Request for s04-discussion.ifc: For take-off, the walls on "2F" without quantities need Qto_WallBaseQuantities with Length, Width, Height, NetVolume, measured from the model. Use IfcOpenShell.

First a look at what the model holds.

```python
import ifcopenshell
import ifcopenshell.util.element
import ifcopenshell.util.unit

model = ifcopenshell.open("s04-discussion.ifc")
print(model.schema)
for unit_type in ("LENGTHUNIT", "AREAUNIT", "VOLUMEUNIT"):
    print(unit_type, ifcopenshell.util.unit.calculate_unit_scale(model, unit_type))
storey = next(s for s in model.by_type("IfcBuildingStorey") if s.Name == "2F")
walls = [e for e in ifcopenshell.util.element.get_decomposition(storey) if e.is_a("IfcWall")]
for e in sorted(walls, key=lambda e: e.id()):
    print(e.id(), e.is_a(), e.Name, list(ifcopenshell.util.element.get_psets(e, qtos_only=True)), sep=" | ")
```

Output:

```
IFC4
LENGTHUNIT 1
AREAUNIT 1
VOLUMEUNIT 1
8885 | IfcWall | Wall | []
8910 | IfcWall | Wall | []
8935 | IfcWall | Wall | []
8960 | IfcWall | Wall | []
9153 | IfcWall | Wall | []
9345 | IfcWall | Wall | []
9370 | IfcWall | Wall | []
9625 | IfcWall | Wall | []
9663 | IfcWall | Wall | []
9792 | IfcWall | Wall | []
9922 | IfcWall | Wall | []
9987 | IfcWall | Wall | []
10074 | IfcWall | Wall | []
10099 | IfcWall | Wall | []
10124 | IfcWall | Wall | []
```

```python
import ifcopenshell
import ifcopenshell.api.pset
import ifcopenshell.geom
import ifcopenshell.util.element
import ifcopenshell.util.shape
import ifcopenshell.util.unit

model = ifcopenshell.open("s04-discussion.ifc")
unit_scale = ifcopenshell.util.unit.calculate_unit_scale(model)
volume_scale = ifcopenshell.util.unit.calculate_unit_scale(model, "VOLUMEUNIT")
settings = ifcopenshell.geom.settings()

storey = next(s for s in model.by_type("IfcBuildingStorey") if s.Name == "2F")
walls = [e for e in ifcopenshell.util.element.get_decomposition(storey) if e.is_a("IfcWall")]

for e in sorted(walls, key=lambda e: e.id()):
    if ifcopenshell.util.element.get_psets(e, qtos_only=True, should_inherit=False):
        continue
    # Geometry comes back in metres, in the element's own axes.
    shape = ifcopenshell.geom.create_shape(settings, e)
    values = {
        "Length": ifcopenshell.util.shape.get_x(shape.geometry) / unit_scale,
        "Width": ifcopenshell.util.shape.get_y(shape.geometry) / unit_scale,
        "Height": ifcopenshell.util.shape.get_z(shape.geometry) / unit_scale,
        "NetVolume": ifcopenshell.util.shape.get_volume(shape.geometry) / volume_scale,
    }
    qto = ifcopenshell.api.pset.add_qto(model, product=e, name="Qto_WallBaseQuantities")
    ifcopenshell.api.pset.edit_qto(model, qto=qto, properties=values)
    print(e.id(), {k: round(v, 3) for k, v in values.items()})

model.write("s04-discussion_updated.ifc")
```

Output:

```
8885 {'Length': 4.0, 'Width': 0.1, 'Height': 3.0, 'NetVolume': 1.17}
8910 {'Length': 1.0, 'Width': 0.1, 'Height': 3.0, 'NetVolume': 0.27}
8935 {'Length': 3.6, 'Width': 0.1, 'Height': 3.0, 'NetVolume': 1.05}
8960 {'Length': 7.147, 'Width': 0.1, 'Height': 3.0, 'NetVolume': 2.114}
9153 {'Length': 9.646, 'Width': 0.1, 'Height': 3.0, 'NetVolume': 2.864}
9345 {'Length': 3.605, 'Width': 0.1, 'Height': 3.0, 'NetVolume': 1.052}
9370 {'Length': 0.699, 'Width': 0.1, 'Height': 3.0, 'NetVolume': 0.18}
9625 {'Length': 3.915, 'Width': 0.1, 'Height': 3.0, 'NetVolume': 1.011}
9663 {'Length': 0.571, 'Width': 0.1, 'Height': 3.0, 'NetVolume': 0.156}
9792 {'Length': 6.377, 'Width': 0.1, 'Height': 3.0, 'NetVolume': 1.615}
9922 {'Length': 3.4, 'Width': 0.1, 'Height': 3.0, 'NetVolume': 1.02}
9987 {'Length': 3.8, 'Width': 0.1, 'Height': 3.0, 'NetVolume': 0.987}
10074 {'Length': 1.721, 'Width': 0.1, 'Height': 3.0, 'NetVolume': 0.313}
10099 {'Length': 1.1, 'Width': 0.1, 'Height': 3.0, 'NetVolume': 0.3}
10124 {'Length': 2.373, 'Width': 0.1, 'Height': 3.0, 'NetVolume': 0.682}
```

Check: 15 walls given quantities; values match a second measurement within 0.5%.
